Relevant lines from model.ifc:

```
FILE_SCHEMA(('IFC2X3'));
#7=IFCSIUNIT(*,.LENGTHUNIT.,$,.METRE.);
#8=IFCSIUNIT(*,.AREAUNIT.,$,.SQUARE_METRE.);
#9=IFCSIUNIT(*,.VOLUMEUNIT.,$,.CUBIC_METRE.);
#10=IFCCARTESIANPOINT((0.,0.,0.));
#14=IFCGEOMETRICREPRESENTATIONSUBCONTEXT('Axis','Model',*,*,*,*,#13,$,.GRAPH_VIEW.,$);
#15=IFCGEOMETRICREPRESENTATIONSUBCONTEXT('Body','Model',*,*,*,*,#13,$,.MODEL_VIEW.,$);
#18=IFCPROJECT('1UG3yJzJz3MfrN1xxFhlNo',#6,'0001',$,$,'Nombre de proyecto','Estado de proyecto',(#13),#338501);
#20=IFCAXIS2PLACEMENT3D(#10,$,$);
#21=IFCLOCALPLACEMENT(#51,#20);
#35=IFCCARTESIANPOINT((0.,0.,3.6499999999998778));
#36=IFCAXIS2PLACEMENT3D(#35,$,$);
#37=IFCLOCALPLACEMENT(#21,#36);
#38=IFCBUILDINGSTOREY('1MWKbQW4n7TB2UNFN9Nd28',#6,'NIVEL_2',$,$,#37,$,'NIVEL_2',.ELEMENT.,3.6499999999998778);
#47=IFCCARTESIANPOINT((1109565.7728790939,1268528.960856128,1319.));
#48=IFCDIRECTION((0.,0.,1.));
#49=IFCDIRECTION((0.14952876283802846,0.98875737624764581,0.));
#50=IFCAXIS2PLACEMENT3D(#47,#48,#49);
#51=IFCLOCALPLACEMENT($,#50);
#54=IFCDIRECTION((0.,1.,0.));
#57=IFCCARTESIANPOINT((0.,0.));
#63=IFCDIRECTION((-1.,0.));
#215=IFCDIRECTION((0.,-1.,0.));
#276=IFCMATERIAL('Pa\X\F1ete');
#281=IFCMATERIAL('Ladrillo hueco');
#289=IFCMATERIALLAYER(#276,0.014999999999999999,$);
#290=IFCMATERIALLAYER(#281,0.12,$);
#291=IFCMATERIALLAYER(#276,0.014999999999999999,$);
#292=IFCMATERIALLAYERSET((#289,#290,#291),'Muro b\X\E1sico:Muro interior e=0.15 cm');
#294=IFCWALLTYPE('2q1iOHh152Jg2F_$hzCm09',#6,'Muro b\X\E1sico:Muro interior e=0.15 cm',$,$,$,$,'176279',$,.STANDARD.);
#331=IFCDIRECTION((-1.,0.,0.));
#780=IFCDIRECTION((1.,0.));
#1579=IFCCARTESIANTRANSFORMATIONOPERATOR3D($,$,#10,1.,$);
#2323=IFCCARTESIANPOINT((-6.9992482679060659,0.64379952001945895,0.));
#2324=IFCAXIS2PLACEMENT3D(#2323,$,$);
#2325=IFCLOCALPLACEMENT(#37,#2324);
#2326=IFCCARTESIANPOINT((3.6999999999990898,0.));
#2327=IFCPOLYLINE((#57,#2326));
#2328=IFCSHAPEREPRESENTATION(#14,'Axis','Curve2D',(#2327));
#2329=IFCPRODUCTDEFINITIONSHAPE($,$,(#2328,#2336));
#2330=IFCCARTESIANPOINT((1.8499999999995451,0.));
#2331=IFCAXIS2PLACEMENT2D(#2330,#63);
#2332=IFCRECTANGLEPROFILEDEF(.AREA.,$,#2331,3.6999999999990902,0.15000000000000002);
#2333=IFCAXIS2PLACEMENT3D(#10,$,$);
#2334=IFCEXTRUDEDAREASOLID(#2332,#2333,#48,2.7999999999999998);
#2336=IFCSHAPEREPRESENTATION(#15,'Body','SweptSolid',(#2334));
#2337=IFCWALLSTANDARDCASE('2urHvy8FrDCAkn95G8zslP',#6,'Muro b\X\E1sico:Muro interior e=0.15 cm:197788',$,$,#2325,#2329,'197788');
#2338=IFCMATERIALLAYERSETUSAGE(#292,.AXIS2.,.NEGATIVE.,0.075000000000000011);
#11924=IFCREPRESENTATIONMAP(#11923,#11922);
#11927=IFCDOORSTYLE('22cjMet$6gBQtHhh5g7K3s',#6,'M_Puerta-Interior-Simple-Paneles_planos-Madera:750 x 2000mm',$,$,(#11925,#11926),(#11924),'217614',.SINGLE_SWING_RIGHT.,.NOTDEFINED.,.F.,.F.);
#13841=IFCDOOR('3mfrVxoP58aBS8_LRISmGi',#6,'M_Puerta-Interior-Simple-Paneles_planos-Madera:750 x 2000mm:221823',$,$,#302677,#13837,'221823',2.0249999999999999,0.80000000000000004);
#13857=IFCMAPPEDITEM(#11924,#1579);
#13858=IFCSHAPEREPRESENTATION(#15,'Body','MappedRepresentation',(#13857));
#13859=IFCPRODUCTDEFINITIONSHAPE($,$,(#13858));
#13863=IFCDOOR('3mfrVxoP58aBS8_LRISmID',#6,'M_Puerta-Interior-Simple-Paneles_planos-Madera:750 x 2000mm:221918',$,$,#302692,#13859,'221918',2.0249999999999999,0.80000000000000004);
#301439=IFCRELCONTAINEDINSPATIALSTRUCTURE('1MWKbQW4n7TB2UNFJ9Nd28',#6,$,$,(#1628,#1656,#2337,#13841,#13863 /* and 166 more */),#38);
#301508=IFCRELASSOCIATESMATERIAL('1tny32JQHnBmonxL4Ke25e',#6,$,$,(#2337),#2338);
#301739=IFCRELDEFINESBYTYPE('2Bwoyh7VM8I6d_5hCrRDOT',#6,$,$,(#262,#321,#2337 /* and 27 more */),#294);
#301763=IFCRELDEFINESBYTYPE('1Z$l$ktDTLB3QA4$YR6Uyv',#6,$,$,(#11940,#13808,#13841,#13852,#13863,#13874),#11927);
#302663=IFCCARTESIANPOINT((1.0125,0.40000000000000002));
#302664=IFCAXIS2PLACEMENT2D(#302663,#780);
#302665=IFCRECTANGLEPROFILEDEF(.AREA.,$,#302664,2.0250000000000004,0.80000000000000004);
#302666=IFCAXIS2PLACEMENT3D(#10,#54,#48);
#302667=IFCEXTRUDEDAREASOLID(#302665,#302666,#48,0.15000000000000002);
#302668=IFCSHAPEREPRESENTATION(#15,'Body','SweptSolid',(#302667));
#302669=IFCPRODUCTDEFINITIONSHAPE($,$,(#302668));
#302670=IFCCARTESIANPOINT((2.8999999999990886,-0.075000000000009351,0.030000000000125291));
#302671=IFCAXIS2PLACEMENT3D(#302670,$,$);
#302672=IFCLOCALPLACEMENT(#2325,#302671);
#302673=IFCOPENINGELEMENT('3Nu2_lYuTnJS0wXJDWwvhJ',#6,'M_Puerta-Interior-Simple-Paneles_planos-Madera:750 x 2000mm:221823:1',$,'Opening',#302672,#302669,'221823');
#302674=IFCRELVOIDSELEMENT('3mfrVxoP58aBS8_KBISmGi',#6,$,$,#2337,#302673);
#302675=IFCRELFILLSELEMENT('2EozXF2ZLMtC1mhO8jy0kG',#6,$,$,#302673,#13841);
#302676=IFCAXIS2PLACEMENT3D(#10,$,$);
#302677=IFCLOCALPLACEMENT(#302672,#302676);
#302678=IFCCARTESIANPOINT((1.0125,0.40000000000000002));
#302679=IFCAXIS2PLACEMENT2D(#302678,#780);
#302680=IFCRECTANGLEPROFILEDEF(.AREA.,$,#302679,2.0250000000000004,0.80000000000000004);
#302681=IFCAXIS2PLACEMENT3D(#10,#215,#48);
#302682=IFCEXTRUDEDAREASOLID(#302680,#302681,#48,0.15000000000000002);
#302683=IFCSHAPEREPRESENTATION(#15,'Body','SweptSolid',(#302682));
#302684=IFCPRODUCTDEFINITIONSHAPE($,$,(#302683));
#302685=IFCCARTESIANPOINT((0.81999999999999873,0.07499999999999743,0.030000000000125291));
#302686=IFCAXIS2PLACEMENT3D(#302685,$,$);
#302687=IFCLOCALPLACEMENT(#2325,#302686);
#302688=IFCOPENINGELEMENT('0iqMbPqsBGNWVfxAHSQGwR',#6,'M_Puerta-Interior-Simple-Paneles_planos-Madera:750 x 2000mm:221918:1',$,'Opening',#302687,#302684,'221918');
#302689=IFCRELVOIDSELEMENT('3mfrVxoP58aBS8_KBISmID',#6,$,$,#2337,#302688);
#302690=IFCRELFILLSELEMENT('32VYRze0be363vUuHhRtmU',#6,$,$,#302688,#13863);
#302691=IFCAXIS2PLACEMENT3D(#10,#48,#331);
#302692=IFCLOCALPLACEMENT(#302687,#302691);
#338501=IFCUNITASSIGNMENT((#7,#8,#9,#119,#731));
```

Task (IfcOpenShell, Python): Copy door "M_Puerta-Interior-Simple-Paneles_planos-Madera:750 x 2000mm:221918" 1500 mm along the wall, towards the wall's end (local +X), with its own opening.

```python
import ifcopenshell
import ifcopenshell.api.feature
import ifcopenshell.api.geometry
import ifcopenshell.api.root
import ifcopenshell.geom
import ifcopenshell.util.element
import ifcopenshell.util.placement
import ifcopenshell.util.shape

model = ifcopenshell.open("model.ifc")
settings = ifcopenshell.geom.settings()


def volume(element):
    """Net volume in cubic metres, openings subtracted."""
    shape = ifcopenshell.geom.create_shape(settings, element)
    return ifcopenshell.util.shape.get_volume(shape.geometry)


def reuse_history(source, copy):
    """copy_class also copies each property set's owner history, people and application; keep the originals."""
    for rel in copy.IsDefinedBy:
        if rel.is_a("IfcRelDefinesByProperties") and (history := rel.RelatingPropertyDefinition.OwnerHistory):
            rel.RelatingPropertyDefinition.OwnerHistory = source.OwnerHistory
            ifcopenshell.util.element.remove_deep2(model, history)


door = model.by_id(13863)
opening = door.FillsVoids[0].RelatingOpeningElement
wall = opening.VoidsElements[0].RelatingBuildingElement
before = volume(wall)
shift = ifcopenshell.util.placement.get_local_placement(wall.ObjectPlacement)[:3, 0] * 1.5

# copy_class copies the void relationship, type, container and properties, but no geometry.
new_opening = ifcopenshell.api.root.copy_class(model, product=opening)
new_opening.Representation = ifcopenshell.util.element.copy_deep(
    model, opening.Representation, exclude=["IfcGeometricRepresentationContext", "IfcRepresentationMap"]
)
new_opening.Name = "M_Puerta-Interior-Simple-Paneles_planos-Madera:750 x 2000mm"
new_opening.Tag = None
new_door = ifcopenshell.api.root.copy_class(model, product=door)
new_door.Representation = ifcopenshell.util.element.copy_deep(
    model, door.Representation, exclude=["IfcGeometricRepresentationContext", "IfcRepresentationMap"]
)
new_door.Name = "M_Puerta-Interior-Simple-Paneles_planos-Madera:750 x 2000mm"
new_door.Tag = None
reuse_history(door, new_door)
fills = ifcopenshell.api.feature.add_filling(model, opening=new_opening, element=new_door)
fills.OwnerHistory = new_door.OwnerHistory  # required in IFC2X3

for old, new in ((opening, new_opening), (door, new_door)):
    matrix = ifcopenshell.util.placement.get_local_placement(old.ObjectPlacement)
    matrix[:3, 3] += shift
    ifcopenshell.api.geometry.edit_object_placement(model, product=new, matrix=matrix, is_si=False)

after = volume(wall)

print(f"wall volume {before:.3f} -> {after:.3f} m3")

model.write("model_edited.ifc")
```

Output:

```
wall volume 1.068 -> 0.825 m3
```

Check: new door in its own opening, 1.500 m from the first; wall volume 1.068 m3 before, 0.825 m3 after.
